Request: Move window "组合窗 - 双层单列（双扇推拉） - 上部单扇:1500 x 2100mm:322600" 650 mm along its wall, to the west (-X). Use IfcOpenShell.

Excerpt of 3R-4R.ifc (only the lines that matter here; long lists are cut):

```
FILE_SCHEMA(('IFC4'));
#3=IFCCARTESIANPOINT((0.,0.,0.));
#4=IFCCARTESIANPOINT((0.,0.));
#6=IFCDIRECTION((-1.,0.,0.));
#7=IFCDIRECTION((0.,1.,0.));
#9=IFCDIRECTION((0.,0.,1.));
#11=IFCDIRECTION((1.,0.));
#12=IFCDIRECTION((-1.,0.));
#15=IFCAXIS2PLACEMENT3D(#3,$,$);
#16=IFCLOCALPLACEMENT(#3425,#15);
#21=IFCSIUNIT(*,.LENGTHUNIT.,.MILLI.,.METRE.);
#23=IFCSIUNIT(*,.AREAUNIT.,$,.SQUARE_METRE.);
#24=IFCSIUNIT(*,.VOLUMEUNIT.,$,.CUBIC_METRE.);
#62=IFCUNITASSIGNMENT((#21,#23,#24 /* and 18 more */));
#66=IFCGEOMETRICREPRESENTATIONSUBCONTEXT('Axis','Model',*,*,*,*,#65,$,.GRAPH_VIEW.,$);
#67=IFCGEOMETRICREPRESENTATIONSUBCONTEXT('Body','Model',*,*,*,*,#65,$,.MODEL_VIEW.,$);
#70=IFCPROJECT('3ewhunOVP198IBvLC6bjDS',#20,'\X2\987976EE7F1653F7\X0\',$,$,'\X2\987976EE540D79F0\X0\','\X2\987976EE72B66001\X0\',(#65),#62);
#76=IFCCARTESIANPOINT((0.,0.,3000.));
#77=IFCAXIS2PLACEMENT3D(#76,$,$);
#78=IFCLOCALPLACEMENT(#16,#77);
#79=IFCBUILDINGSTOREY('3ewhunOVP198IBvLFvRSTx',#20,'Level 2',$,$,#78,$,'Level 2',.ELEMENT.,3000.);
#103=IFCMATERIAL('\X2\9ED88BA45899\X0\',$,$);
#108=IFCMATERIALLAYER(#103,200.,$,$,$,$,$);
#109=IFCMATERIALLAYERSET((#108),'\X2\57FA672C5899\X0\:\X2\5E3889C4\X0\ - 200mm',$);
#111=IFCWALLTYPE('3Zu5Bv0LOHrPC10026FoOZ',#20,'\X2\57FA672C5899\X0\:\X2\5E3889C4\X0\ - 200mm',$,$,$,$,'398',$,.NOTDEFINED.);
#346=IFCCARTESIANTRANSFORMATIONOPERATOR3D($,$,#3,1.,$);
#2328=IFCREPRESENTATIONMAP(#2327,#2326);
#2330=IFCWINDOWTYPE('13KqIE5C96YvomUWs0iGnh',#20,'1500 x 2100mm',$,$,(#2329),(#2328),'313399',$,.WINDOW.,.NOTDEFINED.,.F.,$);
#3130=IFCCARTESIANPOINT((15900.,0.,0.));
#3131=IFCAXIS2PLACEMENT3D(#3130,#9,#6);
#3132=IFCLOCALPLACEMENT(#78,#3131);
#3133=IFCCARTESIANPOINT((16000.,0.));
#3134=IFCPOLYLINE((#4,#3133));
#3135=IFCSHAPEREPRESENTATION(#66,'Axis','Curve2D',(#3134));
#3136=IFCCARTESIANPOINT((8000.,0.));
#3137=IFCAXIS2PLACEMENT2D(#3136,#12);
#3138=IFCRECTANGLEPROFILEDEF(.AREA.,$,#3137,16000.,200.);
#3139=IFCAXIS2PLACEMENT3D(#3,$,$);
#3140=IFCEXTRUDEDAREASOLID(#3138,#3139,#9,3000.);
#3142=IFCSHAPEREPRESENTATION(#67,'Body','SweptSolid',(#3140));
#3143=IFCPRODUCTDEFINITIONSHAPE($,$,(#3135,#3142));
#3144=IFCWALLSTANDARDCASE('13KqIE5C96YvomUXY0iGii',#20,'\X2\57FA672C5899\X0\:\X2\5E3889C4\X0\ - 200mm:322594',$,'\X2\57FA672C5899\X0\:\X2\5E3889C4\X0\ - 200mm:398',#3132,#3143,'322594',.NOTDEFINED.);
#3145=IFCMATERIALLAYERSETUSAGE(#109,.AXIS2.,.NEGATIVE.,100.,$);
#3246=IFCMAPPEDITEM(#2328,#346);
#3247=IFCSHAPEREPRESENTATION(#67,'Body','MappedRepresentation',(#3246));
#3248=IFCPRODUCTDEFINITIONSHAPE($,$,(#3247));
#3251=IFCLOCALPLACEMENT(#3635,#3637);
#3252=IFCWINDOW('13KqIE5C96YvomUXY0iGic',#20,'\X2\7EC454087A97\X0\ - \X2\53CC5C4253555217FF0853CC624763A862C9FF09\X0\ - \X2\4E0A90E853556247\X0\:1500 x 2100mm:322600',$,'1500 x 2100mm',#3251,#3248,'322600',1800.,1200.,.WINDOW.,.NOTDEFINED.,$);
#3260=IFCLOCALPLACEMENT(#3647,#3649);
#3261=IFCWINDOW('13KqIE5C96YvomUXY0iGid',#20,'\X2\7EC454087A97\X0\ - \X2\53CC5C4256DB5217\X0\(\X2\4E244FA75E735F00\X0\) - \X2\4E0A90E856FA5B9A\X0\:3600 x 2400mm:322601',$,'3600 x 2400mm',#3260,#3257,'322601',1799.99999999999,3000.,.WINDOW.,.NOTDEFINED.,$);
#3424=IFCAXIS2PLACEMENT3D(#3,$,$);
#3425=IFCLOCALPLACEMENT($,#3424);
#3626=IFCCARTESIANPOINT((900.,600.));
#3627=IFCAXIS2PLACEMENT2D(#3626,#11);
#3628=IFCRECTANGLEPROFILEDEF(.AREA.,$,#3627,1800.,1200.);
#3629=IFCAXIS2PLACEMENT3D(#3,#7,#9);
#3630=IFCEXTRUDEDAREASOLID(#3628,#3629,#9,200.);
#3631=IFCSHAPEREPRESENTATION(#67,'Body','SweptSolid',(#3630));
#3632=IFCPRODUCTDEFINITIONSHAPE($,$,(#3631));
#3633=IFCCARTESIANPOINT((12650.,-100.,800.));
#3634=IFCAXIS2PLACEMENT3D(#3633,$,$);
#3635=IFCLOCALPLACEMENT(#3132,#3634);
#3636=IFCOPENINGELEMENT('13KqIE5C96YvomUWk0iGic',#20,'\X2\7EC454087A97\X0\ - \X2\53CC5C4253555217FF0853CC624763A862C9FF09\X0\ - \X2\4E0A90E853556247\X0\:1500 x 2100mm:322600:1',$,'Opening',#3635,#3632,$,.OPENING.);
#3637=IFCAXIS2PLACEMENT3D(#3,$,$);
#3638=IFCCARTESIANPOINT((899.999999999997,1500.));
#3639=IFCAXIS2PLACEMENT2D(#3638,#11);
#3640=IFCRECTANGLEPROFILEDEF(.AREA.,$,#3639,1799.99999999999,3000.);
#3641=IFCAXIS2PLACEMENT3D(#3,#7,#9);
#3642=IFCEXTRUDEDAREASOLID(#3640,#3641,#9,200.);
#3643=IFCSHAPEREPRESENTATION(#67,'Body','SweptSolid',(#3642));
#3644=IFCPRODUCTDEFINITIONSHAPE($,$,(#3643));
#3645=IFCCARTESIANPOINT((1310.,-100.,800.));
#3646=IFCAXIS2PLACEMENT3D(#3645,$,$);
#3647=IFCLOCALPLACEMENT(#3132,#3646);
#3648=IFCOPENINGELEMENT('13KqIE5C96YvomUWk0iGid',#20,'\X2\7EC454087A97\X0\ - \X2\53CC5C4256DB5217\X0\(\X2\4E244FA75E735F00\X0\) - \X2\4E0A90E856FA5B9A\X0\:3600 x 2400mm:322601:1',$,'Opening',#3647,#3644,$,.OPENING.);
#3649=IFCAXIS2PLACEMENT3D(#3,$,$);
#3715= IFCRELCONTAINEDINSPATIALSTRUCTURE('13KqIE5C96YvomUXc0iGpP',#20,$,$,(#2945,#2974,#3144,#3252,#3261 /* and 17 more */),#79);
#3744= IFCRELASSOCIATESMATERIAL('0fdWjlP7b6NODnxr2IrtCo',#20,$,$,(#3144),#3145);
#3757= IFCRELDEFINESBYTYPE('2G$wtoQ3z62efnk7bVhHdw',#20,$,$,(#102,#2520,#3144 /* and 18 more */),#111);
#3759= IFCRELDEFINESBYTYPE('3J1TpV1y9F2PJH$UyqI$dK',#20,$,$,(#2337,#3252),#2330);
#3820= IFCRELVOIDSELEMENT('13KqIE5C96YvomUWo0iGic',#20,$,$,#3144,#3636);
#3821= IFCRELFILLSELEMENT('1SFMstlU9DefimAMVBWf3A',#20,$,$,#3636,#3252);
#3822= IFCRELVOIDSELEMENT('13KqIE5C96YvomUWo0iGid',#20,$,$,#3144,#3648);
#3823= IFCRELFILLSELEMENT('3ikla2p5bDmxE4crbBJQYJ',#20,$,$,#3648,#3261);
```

```python
import ifcopenshell
import ifcopenshell.api.geometry
import ifcopenshell.util.placement
import ifcopenshell.util.unit

model = ifcopenshell.open("3R-4R.ifc")
unit_scale = ifcopenshell.util.unit.calculate_unit_scale(model)

window = model.by_guid("13KqIE5C96YvomUXY0iGic")
opening = window.FillsVoids[0].RelatingOpeningElement
wall = opening.VoidsElements[0].RelatingBuildingElement

wall_matrix = ifcopenshell.util.placement.get_local_placement(wall.ObjectPlacement)
shift = wall_matrix[:3, 0] * 0.65 / unit_scale
before = ifcopenshell.util.placement.get_local_placement(window.ObjectPlacement)[:3, 3].copy()

# The window is placed relative to its opening, so it follows when the opening moves.
matrix = ifcopenshell.util.placement.get_local_placement(opening.ObjectPlacement)
matrix[:3, 3] += shift
ifcopenshell.api.geometry.edit_object_placement(
    model, product=opening, matrix=matrix, is_si=False, should_transform_children=True
)

after = ifcopenshell.util.placement.get_local_placement(window.ObjectPlacement)[:3, 3]
print("window moved by", (after - before).round(3) + 0.0)

model.write("3R-4R_rev.ifc")
```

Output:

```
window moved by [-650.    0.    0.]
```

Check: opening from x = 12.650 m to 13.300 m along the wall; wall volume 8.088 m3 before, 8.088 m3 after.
